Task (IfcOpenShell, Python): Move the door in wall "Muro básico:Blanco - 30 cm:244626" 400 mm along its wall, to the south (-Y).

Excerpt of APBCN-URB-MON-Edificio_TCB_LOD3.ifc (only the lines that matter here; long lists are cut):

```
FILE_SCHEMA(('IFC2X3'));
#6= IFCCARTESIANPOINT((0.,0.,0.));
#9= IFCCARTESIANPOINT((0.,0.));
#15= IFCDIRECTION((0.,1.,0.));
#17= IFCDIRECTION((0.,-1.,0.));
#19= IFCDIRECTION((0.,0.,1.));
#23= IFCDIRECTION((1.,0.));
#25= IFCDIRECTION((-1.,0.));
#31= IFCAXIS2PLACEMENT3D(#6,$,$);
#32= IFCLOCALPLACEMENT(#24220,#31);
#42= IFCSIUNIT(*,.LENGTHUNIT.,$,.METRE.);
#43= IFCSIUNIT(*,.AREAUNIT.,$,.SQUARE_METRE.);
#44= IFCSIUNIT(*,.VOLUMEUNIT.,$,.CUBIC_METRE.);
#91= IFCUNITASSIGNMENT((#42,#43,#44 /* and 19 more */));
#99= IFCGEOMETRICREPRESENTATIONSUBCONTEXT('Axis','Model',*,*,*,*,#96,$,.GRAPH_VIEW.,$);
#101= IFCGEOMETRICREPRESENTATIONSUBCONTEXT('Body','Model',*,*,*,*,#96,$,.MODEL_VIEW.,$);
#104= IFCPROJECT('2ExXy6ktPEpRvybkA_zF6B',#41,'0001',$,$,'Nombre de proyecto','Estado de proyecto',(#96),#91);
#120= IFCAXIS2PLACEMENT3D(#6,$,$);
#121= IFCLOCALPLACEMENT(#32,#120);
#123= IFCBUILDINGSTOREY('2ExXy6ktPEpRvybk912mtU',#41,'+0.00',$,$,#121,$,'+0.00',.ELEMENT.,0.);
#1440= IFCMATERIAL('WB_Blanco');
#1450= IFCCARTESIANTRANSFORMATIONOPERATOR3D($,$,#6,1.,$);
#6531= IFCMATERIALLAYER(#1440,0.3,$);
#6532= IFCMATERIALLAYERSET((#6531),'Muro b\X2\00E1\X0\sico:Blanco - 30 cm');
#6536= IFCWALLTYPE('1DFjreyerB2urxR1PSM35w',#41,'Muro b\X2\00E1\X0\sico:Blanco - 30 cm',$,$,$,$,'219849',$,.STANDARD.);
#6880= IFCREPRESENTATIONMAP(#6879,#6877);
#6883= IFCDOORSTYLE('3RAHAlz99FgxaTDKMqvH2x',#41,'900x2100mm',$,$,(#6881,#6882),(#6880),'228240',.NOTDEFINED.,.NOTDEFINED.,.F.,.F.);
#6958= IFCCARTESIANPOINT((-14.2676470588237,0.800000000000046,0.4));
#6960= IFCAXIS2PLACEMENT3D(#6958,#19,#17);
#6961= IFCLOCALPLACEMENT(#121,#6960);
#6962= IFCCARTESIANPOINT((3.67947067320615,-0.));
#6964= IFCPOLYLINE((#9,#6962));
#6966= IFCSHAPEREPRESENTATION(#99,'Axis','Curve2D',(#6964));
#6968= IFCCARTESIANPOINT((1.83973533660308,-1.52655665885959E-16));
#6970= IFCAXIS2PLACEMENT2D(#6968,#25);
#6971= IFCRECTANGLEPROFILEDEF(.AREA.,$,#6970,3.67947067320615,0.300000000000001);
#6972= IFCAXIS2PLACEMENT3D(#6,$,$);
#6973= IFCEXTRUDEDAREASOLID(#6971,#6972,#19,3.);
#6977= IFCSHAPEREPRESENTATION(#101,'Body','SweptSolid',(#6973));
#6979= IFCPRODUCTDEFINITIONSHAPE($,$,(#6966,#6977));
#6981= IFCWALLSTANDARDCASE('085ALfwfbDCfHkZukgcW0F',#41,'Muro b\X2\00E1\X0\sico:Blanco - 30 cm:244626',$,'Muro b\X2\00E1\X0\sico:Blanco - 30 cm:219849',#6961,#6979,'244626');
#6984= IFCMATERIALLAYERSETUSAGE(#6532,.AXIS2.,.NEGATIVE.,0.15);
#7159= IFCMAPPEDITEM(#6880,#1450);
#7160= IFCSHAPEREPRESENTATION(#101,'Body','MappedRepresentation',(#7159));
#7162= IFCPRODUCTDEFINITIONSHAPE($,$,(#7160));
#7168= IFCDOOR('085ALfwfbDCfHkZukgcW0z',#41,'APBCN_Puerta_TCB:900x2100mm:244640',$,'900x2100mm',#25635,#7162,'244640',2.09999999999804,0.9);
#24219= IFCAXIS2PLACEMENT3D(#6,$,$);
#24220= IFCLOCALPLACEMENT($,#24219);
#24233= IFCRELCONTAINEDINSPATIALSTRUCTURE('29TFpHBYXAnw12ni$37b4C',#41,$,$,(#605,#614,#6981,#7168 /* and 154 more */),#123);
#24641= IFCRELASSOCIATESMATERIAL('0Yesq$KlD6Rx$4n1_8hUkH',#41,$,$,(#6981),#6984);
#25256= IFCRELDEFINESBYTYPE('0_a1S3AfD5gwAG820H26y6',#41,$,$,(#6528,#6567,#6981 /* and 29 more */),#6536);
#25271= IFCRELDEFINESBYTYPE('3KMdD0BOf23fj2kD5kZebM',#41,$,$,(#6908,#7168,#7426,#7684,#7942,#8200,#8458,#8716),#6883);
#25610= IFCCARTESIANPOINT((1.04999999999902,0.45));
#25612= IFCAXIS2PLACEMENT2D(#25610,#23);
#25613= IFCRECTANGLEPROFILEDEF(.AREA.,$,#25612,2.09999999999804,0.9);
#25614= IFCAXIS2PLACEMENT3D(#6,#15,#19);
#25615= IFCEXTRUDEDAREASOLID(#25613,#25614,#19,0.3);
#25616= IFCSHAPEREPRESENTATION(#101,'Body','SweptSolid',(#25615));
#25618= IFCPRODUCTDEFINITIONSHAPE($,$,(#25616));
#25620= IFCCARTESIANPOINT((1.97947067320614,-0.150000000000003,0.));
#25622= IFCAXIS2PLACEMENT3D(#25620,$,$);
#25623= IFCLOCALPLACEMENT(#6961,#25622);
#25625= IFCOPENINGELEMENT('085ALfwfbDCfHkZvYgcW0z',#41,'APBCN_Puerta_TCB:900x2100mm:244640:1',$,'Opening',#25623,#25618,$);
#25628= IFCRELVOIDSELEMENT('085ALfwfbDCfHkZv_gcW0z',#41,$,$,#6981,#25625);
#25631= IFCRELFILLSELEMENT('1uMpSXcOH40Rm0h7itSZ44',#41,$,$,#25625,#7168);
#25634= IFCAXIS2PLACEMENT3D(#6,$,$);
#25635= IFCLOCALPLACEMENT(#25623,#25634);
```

```python
import ifcopenshell
import ifcopenshell.api.geometry
import ifcopenshell.util.placement
import ifcopenshell.util.unit

model = ifcopenshell.open("APBCN-URB-MON-Edificio_TCB_LOD3.ifc")
unit_scale = ifcopenshell.util.unit.calculate_unit_scale(model)

door = model.by_guid("085ALfwfbDCfHkZukgcW0z")
opening = door.FillsVoids[0].RelatingOpeningElement
wall = opening.VoidsElements[0].RelatingBuildingElement

wall_matrix = ifcopenshell.util.placement.get_local_placement(wall.ObjectPlacement)
shift = wall_matrix[:3, 0] * 0.4 / unit_scale
before = ifcopenshell.util.placement.get_local_placement(door.ObjectPlacement)[:3, 3].copy()

# The door is placed relative to its opening, so it follows when the opening moves.
matrix = ifcopenshell.util.placement.get_local_placement(opening.ObjectPlacement)
matrix[:3, 3] += shift
ifcopenshell.api.geometry.edit_object_placement(
    model, product=opening, matrix=matrix, is_si=False, should_transform_children=True
)

after = ifcopenshell.util.placement.get_local_placement(door.ObjectPlacement)[:3, 3]
print("door moved by", (after - before).round(3) + 0.0)

model.write("APBCN-URB-MON-Edificio_TCB_LOD3-out.ifc")
```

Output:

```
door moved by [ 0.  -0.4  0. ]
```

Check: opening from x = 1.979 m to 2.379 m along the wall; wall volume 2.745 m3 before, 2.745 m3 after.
